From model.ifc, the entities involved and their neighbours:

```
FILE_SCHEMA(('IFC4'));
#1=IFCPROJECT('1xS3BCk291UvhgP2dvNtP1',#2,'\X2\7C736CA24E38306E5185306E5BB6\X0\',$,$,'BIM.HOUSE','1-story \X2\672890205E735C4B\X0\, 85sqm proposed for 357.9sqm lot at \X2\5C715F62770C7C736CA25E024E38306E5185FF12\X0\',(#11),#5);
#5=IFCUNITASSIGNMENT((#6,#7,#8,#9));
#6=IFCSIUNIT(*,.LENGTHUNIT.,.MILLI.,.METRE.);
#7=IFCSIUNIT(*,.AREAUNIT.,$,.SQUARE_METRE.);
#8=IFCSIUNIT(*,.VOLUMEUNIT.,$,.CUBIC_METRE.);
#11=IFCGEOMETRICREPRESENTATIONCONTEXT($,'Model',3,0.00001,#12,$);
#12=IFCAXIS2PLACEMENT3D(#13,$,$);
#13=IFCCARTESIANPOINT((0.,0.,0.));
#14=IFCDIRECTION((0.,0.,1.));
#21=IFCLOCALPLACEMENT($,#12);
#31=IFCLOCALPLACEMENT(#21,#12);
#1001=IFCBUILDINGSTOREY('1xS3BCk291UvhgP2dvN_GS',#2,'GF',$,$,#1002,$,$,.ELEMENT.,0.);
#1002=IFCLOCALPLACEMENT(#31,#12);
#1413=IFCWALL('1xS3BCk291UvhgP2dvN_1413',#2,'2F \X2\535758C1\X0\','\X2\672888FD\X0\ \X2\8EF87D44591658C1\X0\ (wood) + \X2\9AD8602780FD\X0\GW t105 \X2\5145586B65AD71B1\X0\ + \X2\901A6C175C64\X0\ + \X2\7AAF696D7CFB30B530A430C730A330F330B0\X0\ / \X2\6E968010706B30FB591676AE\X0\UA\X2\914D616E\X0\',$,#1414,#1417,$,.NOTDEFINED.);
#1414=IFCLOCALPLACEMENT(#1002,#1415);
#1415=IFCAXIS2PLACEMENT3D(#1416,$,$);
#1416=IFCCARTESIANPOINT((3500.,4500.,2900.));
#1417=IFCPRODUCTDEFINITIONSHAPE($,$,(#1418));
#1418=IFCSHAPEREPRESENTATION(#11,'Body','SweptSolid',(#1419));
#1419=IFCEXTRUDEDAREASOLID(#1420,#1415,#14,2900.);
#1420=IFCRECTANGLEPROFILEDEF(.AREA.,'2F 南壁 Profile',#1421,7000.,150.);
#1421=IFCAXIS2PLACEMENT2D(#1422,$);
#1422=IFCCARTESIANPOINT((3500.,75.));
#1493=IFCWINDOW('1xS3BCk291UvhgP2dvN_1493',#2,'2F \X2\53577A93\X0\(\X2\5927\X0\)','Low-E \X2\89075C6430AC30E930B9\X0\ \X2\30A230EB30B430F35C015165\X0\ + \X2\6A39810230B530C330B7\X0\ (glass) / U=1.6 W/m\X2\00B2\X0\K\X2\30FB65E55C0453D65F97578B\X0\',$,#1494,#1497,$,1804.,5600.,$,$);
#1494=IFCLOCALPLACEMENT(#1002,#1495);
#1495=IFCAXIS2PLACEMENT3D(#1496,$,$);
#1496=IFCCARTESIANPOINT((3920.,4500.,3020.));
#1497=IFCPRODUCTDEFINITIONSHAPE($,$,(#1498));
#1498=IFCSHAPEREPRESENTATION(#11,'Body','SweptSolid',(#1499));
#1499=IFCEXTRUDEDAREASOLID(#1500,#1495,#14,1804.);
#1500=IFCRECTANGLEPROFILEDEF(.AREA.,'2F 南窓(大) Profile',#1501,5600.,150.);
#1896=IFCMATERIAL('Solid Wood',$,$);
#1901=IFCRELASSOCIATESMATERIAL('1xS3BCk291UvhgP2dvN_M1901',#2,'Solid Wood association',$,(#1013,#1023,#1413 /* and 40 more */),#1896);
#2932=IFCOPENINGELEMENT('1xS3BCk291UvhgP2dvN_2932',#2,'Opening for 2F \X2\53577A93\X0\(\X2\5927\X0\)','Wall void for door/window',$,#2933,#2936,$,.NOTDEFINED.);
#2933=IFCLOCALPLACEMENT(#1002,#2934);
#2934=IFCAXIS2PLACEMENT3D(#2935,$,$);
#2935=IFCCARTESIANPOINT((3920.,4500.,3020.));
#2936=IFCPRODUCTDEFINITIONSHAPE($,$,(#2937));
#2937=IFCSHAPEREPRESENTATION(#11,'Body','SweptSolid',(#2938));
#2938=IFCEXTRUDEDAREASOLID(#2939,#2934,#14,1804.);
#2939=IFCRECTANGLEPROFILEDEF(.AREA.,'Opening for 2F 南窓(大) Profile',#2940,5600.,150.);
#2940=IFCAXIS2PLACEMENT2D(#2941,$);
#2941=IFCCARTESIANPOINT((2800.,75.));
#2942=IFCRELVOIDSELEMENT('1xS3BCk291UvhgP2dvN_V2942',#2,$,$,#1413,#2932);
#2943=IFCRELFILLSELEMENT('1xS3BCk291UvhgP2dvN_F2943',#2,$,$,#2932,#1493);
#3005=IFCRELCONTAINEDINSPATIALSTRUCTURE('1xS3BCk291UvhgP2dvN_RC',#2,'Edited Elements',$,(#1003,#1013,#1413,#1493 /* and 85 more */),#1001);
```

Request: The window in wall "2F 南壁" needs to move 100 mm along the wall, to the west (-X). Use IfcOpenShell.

```python
import ifcopenshell
import ifcopenshell.api.geometry
import ifcopenshell.util.placement
import ifcopenshell.util.unit

model = ifcopenshell.open("model.ifc")
unit_scale = ifcopenshell.util.unit.calculate_unit_scale(model)

window = model.by_guid("1xS3BCk291UvhgP2dvN_1493")
opening = window.FillsVoids[0].RelatingOpeningElement
wall = opening.VoidsElements[0].RelatingBuildingElement

wall_matrix = ifcopenshell.util.placement.get_local_placement(wall.ObjectPlacement)
shift = wall_matrix[:3, 0] * -0.1 / unit_scale
before = ifcopenshell.util.placement.get_local_placement(window.ObjectPlacement)[:3, 3].copy()

# The window is not placed relative to its opening, so move both.
for product in (opening, window):
    matrix = ifcopenshell.util.placement.get_local_placement(product.ObjectPlacement)
    matrix[:3, 3] += shift
    ifcopenshell.api.geometry.edit_object_placement(model, product=product, matrix=matrix, is_si=False)

after = ifcopenshell.util.placement.get_local_placement(window.ObjectPlacement)[:3, 3]
print("window moved by", (after - before).round(3) + 0.0)

model.write("model_edited.ifc")
```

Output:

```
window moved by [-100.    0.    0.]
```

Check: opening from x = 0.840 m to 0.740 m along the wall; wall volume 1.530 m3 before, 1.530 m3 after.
